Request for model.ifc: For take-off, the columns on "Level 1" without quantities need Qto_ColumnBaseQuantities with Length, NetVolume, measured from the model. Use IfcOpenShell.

First a look at what the model holds.

```python
import ifcopenshell
import ifcopenshell.util.element
import ifcopenshell.util.unit

model = ifcopenshell.open("model.ifc")
print(model.schema)
for unit_type in ("LENGTHUNIT", "AREAUNIT", "VOLUMEUNIT"):
    print(unit_type, ifcopenshell.util.unit.calculate_unit_scale(model, unit_type))
storey = next(s for s in model.by_type("IfcBuildingStorey") if s.Name == "Level 1")
columns = [e for e in ifcopenshell.util.element.get_decomposition(storey) if e.is_a("IfcColumn")]
for e in sorted(columns, key=lambda e: e.id()):
    print(e.id(), e.is_a(), e.Name, list(ifcopenshell.util.element.get_psets(e, qtos_only=True)), sep=" | ")
```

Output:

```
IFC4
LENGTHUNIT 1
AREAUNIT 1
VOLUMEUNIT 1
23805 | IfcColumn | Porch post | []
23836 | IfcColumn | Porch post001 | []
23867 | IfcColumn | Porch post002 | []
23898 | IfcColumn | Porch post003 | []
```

```python
import ifcopenshell
import ifcopenshell.api.pset
import ifcopenshell.geom
import ifcopenshell.util.element
import ifcopenshell.util.shape
import ifcopenshell.util.unit

model = ifcopenshell.open("model.ifc")
unit_scale = ifcopenshell.util.unit.calculate_unit_scale(model)
volume_scale = ifcopenshell.util.unit.calculate_unit_scale(model, "VOLUMEUNIT")
settings = ifcopenshell.geom.settings()

storey = next(s for s in model.by_type("IfcBuildingStorey") if s.Name == "Level 1")
columns = [e for e in ifcopenshell.util.element.get_decomposition(storey) if e.is_a("IfcColumn")]

for e in sorted(columns, key=lambda e: e.id()):
    if ifcopenshell.util.element.get_psets(e, qtos_only=True, should_inherit=False):
        continue
    # Geometry comes back in metres, in the element's own axes.
    shape = ifcopenshell.geom.create_shape(settings, e)
    values = {
        "Length": ifcopenshell.util.shape.get_z(shape.geometry) / unit_scale,
        "NetVolume": ifcopenshell.util.shape.get_volume(shape.geometry) / volume_scale,
    }
    qto = ifcopenshell.api.pset.add_qto(model, product=e, name="Qto_ColumnBaseQuantities")
    ifcopenshell.api.pset.edit_qto(model, qto=qto, properties=values)
    print(e.id(), {k: round(v, 3) for k, v in values.items()})

model.write("model_rev.ifc")
```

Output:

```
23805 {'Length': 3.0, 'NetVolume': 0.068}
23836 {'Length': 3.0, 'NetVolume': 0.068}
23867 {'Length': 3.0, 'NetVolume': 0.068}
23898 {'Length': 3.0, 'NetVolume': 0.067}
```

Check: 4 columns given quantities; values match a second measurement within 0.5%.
